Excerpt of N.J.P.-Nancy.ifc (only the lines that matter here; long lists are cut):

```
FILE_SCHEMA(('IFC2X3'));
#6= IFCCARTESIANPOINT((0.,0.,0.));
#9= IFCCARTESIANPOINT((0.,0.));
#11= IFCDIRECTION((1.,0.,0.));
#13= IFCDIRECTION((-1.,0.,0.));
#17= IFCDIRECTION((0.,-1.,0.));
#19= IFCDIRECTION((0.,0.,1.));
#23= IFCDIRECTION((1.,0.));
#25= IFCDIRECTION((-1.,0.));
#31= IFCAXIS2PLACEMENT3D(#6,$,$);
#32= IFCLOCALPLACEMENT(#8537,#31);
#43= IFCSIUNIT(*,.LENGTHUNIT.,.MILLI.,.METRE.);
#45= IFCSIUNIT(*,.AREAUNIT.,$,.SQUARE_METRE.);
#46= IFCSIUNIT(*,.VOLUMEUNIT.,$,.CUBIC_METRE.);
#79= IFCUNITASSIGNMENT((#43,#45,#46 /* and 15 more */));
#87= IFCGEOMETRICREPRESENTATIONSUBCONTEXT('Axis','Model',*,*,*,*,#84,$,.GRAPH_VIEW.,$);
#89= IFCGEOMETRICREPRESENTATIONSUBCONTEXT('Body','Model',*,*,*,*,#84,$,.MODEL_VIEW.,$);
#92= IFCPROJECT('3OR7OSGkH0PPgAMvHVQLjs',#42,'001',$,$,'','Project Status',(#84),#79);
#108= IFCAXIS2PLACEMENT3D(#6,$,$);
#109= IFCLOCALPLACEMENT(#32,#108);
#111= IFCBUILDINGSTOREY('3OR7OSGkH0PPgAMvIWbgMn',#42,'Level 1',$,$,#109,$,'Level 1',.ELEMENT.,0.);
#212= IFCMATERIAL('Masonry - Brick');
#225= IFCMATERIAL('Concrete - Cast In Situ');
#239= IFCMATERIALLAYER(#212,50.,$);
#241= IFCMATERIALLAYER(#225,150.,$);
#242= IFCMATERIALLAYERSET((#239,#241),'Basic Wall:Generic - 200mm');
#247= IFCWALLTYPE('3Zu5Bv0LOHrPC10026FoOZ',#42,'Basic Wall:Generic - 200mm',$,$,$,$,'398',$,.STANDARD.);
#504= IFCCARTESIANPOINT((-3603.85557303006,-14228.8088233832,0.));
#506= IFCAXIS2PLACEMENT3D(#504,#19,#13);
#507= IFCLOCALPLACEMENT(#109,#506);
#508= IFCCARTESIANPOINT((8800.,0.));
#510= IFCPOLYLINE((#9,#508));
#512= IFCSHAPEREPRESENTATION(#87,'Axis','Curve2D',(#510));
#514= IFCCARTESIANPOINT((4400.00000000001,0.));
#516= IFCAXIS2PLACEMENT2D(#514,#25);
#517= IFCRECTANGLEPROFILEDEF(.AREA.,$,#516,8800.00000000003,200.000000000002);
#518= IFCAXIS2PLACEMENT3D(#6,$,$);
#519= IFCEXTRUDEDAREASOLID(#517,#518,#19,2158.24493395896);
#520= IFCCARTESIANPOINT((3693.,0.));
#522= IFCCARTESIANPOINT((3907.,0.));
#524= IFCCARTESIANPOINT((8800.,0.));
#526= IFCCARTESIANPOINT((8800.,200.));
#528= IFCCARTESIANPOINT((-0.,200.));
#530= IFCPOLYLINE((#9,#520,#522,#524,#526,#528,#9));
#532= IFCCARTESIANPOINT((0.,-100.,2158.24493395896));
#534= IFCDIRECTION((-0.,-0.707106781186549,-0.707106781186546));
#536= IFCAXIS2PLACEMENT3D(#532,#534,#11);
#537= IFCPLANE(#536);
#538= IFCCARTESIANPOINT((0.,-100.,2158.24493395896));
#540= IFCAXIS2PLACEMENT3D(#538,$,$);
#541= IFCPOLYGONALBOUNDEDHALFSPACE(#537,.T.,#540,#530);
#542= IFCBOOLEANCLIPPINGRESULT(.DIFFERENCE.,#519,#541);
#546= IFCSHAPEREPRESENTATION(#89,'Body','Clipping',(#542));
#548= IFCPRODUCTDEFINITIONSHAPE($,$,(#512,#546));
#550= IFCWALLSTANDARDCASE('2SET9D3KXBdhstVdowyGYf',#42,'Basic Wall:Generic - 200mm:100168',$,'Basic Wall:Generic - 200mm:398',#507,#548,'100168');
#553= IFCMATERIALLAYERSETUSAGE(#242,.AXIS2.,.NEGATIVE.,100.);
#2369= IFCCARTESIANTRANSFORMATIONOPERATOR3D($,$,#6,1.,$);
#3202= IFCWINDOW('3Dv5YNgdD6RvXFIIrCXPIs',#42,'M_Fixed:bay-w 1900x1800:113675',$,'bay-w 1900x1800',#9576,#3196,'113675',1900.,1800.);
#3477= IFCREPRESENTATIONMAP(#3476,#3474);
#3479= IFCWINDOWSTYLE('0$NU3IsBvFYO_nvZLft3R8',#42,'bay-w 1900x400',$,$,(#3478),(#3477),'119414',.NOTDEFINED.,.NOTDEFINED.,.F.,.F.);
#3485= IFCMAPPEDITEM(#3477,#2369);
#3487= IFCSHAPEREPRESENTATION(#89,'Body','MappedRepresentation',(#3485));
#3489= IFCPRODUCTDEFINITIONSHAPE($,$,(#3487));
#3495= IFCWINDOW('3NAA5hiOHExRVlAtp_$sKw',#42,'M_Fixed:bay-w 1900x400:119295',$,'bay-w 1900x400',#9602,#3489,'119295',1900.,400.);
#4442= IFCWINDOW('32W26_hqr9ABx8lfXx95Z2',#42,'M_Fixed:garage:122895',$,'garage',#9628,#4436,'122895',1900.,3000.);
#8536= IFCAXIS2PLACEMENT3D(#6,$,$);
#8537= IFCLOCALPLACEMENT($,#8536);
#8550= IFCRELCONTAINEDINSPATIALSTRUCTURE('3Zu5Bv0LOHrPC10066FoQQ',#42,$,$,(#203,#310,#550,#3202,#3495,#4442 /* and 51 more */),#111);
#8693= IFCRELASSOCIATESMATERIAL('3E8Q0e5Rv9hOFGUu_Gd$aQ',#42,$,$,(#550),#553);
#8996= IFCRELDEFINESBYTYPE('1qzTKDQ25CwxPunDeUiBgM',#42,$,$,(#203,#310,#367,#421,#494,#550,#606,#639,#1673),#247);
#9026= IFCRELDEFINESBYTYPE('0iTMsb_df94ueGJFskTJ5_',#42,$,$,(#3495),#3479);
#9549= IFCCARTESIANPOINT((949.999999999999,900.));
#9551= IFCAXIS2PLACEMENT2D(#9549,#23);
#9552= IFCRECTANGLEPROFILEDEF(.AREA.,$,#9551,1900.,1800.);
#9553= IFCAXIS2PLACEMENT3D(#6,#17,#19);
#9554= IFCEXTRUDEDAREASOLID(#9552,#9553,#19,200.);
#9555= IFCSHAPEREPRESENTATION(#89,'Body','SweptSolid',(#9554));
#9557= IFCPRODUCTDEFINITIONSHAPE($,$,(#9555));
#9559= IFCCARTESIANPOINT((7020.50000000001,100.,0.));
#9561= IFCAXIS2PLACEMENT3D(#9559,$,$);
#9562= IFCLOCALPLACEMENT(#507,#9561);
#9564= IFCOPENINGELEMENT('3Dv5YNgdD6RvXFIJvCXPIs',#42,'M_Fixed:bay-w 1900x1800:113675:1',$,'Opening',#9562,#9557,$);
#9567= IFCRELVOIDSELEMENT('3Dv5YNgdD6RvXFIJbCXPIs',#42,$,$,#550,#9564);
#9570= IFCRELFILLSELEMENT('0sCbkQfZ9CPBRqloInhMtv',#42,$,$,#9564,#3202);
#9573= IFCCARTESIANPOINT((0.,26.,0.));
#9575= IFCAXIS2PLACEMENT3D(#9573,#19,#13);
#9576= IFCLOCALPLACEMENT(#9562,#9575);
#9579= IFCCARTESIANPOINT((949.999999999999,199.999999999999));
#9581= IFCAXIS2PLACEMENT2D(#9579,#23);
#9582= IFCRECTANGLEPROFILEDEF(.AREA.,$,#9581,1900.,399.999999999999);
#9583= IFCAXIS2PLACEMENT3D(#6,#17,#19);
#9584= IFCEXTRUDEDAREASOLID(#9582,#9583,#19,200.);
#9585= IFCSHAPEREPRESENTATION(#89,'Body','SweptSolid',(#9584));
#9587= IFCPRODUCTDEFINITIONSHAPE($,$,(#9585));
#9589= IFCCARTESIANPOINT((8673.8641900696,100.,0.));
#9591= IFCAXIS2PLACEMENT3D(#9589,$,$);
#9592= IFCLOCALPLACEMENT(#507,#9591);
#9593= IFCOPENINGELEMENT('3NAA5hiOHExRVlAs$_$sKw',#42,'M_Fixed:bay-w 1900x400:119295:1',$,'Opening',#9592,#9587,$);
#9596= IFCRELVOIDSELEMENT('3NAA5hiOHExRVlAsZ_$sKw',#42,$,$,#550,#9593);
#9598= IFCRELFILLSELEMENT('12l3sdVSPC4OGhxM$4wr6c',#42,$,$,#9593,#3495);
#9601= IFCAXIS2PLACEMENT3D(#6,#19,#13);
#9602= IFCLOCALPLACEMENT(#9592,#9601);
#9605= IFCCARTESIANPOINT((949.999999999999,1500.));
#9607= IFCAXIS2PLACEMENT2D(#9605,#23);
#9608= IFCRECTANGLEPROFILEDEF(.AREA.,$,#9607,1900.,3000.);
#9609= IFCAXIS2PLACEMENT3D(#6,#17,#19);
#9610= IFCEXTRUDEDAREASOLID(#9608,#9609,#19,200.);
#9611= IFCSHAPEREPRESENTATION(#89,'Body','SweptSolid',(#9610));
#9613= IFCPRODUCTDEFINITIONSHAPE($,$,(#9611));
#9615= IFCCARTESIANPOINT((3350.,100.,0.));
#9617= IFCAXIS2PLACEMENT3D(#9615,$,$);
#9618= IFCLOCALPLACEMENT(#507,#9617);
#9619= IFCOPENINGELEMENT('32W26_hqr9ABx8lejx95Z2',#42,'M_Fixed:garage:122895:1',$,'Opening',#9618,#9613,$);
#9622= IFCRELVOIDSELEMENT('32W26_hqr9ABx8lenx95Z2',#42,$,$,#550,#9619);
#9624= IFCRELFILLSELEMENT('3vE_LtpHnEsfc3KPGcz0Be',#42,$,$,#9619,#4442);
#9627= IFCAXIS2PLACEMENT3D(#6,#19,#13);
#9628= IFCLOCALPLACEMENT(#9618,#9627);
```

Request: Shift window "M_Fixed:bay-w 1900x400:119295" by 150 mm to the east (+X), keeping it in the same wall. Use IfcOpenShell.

```python
import ifcopenshell
import ifcopenshell.api.geometry
import ifcopenshell.util.placement

model = ifcopenshell.open("N.J.P.-Nancy.ifc")

window = model.by_guid("3NAA5hiOHExRVlAtp_$sKw")
opening = window.FillsVoids[0].RelatingOpeningElement
wall = opening.VoidsElements[0].RelatingBuildingElement

wall_matrix = ifcopenshell.util.placement.get_local_placement(wall.ObjectPlacement)
shift = wall_matrix[:3, 0] * -150.0
before = ifcopenshell.util.placement.get_local_placement(window.ObjectPlacement)[:3, 3].copy()

# The window is placed relative to its opening, so it follows when the opening moves.
matrix = ifcopenshell.util.placement.get_local_placement(opening.ObjectPlacement)
matrix[:3, 3] += shift
ifcopenshell.api.geometry.edit_object_placement(
    model, product=opening, matrix=matrix, is_si=False, should_transform_children=True
)

after = ifcopenshell.util.placement.get_local_placement(window.ObjectPlacement)[:3, 3]
print("window moved by", (after - before).round(3) + 0.0)

model.write("N.J.P.-Nancy_edited.ifc")
```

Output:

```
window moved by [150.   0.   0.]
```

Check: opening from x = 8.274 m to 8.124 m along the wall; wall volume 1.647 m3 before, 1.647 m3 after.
